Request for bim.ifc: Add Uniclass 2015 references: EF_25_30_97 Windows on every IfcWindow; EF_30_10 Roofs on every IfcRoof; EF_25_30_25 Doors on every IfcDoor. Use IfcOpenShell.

First a look at what the model holds.

```python
import ifcopenshell

model = ifcopenshell.open("bim.ifc")
print(model.schema)
print("classifications:", [c.Name for c in model.by_type("IfcClassification")])
for ifc_class in ("IfcDoor", "IfcRoof", "IfcStair", "IfcWall", "IfcWindow"):
    print(ifc_class, len(model.by_type(ifc_class)))
```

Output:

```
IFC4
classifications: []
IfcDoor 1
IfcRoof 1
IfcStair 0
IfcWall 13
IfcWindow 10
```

```python
import ifcopenshell
import ifcopenshell.api.classification

model = ifcopenshell.open("bim.ifc")

system = ifcopenshell.api.classification.add_classification(model, classification="Uniclass 2015")

codes = {
    "IfcWindow": ("EF_25_30_97", "Windows"),
    "IfcRoof": ("EF_30_10", "Roofs"),
    "IfcDoor": ("EF_25_30_25", "Doors"),
}
for ifc_class, (code, name) in codes.items():
    products = model.by_type(ifc_class)
    ifcopenshell.api.classification.add_reference(
        model, products=products, classification=system, identification=code, name=name
    )
    print(code, len(products))

model.write("bim-out.ifc")
```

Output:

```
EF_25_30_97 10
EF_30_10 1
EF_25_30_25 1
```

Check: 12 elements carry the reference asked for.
